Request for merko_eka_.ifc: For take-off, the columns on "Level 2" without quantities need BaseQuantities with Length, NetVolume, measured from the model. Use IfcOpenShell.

First a look at what the model holds.

```python
import ifcopenshell
import ifcopenshell.util.element
import ifcopenshell.util.unit

model = ifcopenshell.open("merko_eka_.ifc")
print(model.schema)
for unit_type in ("LENGTHUNIT", "AREAUNIT", "VOLUMEUNIT"):
    print(unit_type, ifcopenshell.util.unit.calculate_unit_scale(model, unit_type))
storey = next(s for s in model.by_type("IfcBuildingStorey") if s.Name == "Level 2")
columns = [e for e in ifcopenshell.util.element.get_decomposition(storey) if e.is_a("IfcColumn")]
for e in sorted(columns, key=lambda e: e.id()):
    print(e.id(), e.is_a(), e.Name, list(ifcopenshell.util.element.get_psets(e, qtos_only=True)), sep=" | ")
```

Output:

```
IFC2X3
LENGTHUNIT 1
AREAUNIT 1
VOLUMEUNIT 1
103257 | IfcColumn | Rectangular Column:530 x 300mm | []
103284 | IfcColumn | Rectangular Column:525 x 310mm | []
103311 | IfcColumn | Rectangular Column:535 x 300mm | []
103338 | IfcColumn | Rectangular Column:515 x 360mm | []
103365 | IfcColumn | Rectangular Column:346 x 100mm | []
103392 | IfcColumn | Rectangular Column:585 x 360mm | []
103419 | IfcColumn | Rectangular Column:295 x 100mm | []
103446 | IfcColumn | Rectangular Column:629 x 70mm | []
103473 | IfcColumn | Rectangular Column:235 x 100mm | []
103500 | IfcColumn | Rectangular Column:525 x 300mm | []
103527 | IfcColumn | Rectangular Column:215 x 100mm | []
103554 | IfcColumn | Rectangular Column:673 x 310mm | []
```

```python
import ifcopenshell
import ifcopenshell.api.pset
import ifcopenshell.geom
import ifcopenshell.util.element
import ifcopenshell.util.shape
import ifcopenshell.util.unit

model = ifcopenshell.open("merko_eka_.ifc")
unit_scale = ifcopenshell.util.unit.calculate_unit_scale(model)
volume_scale = ifcopenshell.util.unit.calculate_unit_scale(model, "VOLUMEUNIT")
settings = ifcopenshell.geom.settings()

storey = next(s for s in model.by_type("IfcBuildingStorey") if s.Name == "Level 2")
columns = [e for e in ifcopenshell.util.element.get_decomposition(storey) if e.is_a("IfcColumn")]

for e in sorted(columns, key=lambda e: e.id()):
    if ifcopenshell.util.element.get_psets(e, qtos_only=True, should_inherit=False):
        continue
    # Geometry comes back in metres, in the element's own axes.
    shape = ifcopenshell.geom.create_shape(settings, e)
    values = {
        "Length": ifcopenshell.util.shape.get_z(shape.geometry) / unit_scale,
        "NetVolume": ifcopenshell.util.shape.get_volume(shape.geometry) / volume_scale,
    }
    qto = ifcopenshell.api.pset.add_qto(model, product=e, name="BaseQuantities")
    ifcopenshell.api.pset.edit_qto(model, qto=qto, properties=values)
    print(e.id(), {k: round(v, 3) for k, v in values.items()})

model.write("merko_eka_-out.ifc")
```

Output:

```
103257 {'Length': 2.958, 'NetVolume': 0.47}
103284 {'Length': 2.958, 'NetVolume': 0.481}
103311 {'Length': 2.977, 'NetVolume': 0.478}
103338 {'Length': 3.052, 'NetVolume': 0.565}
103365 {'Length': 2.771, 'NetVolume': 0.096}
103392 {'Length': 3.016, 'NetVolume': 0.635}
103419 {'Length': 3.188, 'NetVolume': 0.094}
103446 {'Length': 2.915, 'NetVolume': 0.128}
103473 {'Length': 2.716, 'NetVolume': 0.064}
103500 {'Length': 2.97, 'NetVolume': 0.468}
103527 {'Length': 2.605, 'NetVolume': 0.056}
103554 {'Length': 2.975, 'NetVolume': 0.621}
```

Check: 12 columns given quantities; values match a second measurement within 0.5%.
